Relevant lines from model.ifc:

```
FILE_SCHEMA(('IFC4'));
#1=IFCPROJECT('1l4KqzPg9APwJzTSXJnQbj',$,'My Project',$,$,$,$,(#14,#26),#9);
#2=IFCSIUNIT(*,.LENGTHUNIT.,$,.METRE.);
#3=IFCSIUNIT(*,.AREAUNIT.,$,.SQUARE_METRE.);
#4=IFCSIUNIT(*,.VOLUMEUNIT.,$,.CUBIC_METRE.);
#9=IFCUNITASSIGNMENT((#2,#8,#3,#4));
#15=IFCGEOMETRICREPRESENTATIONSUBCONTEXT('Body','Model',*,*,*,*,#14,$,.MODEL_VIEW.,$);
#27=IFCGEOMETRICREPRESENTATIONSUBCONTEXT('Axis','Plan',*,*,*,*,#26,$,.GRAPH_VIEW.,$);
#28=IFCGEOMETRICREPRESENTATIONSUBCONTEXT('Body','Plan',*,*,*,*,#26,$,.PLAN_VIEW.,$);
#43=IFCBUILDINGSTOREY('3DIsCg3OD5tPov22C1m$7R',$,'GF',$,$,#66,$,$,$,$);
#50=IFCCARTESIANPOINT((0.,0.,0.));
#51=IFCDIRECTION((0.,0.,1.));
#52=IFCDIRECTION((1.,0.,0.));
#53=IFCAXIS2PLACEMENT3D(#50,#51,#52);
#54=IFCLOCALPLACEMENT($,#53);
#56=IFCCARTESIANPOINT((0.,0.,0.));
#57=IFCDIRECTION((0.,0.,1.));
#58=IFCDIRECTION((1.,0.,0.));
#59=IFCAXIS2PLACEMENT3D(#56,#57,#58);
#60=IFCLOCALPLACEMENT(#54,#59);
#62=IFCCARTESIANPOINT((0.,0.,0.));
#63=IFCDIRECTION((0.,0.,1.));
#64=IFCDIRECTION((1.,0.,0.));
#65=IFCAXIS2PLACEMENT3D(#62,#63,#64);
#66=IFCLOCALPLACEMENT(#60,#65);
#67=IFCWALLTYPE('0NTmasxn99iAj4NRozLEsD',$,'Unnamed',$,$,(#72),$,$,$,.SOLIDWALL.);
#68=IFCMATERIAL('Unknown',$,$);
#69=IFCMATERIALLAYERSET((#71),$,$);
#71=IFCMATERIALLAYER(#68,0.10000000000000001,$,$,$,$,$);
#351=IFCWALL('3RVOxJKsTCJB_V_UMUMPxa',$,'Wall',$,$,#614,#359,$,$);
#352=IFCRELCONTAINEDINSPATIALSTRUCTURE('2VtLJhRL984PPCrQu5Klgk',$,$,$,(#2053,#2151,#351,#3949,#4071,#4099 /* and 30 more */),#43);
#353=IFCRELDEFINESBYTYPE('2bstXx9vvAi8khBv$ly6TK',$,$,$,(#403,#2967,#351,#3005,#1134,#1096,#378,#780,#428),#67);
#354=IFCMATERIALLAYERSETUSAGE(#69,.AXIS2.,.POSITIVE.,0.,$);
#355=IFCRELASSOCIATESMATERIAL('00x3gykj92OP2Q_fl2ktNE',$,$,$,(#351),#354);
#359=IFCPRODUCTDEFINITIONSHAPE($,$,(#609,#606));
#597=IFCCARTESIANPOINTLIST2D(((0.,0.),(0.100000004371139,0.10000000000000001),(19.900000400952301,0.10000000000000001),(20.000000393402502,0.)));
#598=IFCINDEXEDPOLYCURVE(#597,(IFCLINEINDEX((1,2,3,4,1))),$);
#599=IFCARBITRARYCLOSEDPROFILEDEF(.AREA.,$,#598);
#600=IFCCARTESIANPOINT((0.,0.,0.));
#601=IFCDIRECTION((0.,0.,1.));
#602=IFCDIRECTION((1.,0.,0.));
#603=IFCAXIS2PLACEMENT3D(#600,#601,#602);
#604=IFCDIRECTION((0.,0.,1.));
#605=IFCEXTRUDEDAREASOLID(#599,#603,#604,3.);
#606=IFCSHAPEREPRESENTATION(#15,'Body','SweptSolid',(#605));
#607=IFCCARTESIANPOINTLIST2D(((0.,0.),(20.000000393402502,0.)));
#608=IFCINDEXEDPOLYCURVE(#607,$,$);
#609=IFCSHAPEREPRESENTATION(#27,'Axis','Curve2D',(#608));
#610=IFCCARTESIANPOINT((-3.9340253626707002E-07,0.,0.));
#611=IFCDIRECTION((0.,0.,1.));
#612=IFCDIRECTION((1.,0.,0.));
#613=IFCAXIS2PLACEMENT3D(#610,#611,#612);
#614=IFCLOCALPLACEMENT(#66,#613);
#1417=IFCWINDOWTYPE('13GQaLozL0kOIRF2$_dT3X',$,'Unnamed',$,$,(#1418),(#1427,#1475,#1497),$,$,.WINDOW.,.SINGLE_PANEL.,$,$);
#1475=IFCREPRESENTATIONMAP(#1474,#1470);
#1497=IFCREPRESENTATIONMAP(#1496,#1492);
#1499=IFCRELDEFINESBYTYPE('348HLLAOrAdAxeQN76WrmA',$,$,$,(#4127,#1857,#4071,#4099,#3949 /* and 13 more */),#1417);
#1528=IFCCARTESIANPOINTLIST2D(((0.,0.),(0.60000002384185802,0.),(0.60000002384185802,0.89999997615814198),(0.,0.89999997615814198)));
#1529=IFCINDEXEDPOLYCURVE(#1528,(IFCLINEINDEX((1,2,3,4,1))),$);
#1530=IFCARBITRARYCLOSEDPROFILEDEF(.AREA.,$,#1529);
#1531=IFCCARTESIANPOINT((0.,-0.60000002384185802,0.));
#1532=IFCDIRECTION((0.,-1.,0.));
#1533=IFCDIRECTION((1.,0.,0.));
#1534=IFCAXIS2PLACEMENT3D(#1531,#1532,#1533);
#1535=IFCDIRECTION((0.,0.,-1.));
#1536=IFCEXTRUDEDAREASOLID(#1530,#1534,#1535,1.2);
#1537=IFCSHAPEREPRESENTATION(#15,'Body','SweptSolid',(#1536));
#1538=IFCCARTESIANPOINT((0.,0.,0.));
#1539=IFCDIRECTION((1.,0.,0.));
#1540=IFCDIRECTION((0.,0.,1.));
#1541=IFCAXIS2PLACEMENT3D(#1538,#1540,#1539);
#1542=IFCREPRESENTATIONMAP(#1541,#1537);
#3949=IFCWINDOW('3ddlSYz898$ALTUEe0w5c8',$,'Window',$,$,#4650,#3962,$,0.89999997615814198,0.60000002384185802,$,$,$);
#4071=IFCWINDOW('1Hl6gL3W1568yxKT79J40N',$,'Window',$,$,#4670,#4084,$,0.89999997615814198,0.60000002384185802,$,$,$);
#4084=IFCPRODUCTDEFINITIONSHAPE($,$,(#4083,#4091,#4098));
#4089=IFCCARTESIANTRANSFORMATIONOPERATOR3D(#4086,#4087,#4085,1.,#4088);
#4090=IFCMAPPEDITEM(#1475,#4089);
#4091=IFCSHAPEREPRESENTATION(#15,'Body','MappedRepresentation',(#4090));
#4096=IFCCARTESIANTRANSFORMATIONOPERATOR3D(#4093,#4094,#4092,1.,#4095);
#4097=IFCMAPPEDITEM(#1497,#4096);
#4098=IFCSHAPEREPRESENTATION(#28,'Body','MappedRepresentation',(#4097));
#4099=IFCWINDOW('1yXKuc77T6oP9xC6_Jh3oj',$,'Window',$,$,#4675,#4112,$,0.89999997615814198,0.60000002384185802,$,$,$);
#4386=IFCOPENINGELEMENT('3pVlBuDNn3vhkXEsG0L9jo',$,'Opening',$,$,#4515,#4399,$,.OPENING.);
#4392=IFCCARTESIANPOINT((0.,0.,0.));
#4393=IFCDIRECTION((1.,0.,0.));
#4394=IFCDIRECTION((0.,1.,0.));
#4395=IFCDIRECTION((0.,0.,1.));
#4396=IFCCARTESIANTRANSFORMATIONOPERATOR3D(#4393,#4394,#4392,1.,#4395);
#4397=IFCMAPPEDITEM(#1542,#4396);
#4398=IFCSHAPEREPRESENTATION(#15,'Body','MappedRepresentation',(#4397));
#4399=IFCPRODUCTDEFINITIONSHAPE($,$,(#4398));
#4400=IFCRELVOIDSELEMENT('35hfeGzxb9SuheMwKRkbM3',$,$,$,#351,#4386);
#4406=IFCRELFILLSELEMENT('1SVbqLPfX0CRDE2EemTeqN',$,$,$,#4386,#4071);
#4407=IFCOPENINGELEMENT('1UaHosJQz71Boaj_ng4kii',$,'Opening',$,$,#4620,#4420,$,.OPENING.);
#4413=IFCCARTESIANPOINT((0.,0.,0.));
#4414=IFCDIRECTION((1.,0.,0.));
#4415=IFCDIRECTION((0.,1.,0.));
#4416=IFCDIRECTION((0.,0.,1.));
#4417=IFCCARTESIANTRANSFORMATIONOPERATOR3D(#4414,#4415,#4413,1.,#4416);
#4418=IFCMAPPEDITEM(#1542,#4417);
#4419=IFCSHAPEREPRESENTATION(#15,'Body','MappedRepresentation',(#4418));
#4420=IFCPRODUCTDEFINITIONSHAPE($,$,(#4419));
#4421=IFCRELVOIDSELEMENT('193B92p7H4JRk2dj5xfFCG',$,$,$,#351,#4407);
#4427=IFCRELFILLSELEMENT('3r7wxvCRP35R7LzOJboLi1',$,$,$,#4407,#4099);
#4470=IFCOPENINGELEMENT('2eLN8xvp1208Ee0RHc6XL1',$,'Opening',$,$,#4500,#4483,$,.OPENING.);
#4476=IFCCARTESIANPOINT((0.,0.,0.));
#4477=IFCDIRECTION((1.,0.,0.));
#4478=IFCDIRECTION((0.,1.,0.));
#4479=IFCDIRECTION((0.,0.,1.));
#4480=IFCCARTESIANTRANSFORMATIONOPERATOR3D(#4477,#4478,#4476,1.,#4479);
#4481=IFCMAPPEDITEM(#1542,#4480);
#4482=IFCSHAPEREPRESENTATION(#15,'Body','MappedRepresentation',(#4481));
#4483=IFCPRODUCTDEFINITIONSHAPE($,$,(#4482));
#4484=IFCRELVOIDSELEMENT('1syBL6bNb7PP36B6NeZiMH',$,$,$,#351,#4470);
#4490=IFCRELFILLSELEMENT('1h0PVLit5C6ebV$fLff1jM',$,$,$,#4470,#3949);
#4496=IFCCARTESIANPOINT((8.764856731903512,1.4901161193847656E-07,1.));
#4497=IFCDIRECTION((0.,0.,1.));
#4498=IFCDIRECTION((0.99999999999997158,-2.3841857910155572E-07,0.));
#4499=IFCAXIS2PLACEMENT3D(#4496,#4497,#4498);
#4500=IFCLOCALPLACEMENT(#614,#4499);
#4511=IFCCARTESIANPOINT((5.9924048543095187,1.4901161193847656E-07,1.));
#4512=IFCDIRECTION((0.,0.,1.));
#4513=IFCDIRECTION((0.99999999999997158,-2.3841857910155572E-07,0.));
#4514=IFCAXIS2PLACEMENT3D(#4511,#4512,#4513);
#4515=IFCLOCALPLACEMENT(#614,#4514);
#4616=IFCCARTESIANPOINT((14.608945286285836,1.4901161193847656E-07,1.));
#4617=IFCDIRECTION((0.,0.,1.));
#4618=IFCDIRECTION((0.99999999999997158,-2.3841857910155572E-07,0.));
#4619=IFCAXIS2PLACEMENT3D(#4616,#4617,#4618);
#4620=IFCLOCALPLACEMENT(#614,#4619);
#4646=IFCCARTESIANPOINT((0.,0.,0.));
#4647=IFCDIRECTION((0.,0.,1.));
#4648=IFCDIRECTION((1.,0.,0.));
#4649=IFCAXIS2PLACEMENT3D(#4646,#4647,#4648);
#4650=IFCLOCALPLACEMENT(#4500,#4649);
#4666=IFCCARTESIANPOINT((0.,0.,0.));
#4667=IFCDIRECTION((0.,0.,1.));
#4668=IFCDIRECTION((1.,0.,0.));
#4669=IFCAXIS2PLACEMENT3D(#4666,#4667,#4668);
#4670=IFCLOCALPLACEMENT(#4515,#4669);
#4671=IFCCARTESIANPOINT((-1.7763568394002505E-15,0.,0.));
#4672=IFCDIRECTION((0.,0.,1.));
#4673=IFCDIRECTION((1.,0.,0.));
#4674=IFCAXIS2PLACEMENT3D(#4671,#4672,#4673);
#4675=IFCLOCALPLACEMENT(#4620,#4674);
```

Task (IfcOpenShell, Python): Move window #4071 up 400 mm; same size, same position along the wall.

```python
import numpy as np
import ifcopenshell
import ifcopenshell.api.geometry
import ifcopenshell.util.placement
import ifcopenshell.util.unit

model = ifcopenshell.open("model.ifc")
unit_scale = ifcopenshell.util.unit.calculate_unit_scale(model)

window = model.by_id(4071)
opening = window.FillsVoids[0].RelatingOpeningElement
dz = 0.4

shift = np.array([0.0, 0.0, dz])
# The window is placed relative to its opening, so it follows when the opening moves.
matrix = ifcopenshell.util.placement.get_local_placement(opening.ObjectPlacement)
matrix[:3, 3] += shift
ifcopenshell.api.geometry.edit_object_placement(
    model, product=opening, matrix=matrix, is_si=False, should_transform_children=True
)

print(f"moved by {dz * unit_scale:+.3f} m")

model.write("model-out.ifc")
```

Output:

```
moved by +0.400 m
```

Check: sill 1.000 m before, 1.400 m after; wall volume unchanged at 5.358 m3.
